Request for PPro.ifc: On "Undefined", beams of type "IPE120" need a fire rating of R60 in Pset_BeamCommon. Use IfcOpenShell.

First a look at what the model holds.

```python
import ifcopenshell
import ifcopenshell.util.element

model = ifcopenshell.open("PPro.ifc")
print(model.schema)
storey = next(s for s in model.by_type("IfcBuildingStorey") if s.Name == "Undefined")
beams = [e for e in ifcopenshell.util.element.get_decomposition(storey) if e.is_a("IfcBeam")]
seen = {}
for e in beams:
    element_type = ifcopenshell.util.element.get_type(e)
    key = (element_type.Name if element_type != e and element_type else None, ifcopenshell.util.element.get_pset(e, "Pset_BeamCommon", "FireRating"))
    seen[key] = seen.get(key, 0) + 1
for (name, value), count in sorted(seen.items(), key=str):
    print(count, "x", name, "|", value)
```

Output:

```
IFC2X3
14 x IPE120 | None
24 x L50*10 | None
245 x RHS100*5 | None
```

```python
import ifcopenshell
import ifcopenshell.api.pset
import ifcopenshell.util.element

model = ifcopenshell.open("PPro.ifc")

storey = next(s for s in model.by_type("IfcBuildingStorey") if s.Name == "Undefined")
beams = [e for e in ifcopenshell.util.element.get_decomposition(storey) if e.is_a("IfcBeam")]

count = 0
for e in beams:
    element_type = ifcopenshell.util.element.get_type(e)
    if element_type in (None, e) or element_type.Name != "IPE120":
        continue
    # add_pset returns the element's existing set when there is one.
    pset = ifcopenshell.api.pset.add_pset(model, product=e, name="Pset_BeamCommon")
    ifcopenshell.api.pset.edit_pset(model, pset=pset, properties={"FireRating": "R60"})
    count += 1

print(count, "beams updated")

model.write("PPro_updated.ifc")
```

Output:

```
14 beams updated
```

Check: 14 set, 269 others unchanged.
